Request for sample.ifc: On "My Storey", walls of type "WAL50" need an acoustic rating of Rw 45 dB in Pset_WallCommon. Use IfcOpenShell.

First a look at what the model holds.

```python
import ifcopenshell
import ifcopenshell.util.element

model = ifcopenshell.open("sample.ifc")
print(model.schema)
storey = next(s for s in model.by_type("IfcBuildingStorey") if s.Name == "My Storey")
walls = [e for e in ifcopenshell.util.element.get_decomposition(storey) if e.is_a("IfcWall")]
seen = {}
for e in walls:
    element_type = ifcopenshell.util.element.get_type(e)
    key = (element_type.Name if element_type != e and element_type else None, ifcopenshell.util.element.get_pset(e, "Pset_WallCommon", "AcousticRating"))
    seen[key] = seen.get(key, 0) + 1
for (name, value), count in sorted(seen.items(), key=str):
    print(count, "x", name, "|", value)
```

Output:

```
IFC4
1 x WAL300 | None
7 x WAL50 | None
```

```python
import ifcopenshell
import ifcopenshell.api.pset
import ifcopenshell.util.element

model = ifcopenshell.open("sample.ifc")

storey = next(s for s in model.by_type("IfcBuildingStorey") if s.Name == "My Storey")
walls = [e for e in ifcopenshell.util.element.get_decomposition(storey) if e.is_a("IfcWall")]

count = 0
for e in walls:
    element_type = ifcopenshell.util.element.get_type(e)
    if element_type in (None, e) or element_type.Name != "WAL50":
        continue
    # add_pset returns the element's existing set when there is one.
    pset = ifcopenshell.api.pset.add_pset(model, product=e, name="Pset_WallCommon")
    ifcopenshell.api.pset.edit_pset(model, pset=pset, properties={"AcousticRating": "Rw 45 dB"})
    count += 1

print(count, "walls updated")

model.write("sample_updated.ifc")
```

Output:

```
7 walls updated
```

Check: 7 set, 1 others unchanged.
